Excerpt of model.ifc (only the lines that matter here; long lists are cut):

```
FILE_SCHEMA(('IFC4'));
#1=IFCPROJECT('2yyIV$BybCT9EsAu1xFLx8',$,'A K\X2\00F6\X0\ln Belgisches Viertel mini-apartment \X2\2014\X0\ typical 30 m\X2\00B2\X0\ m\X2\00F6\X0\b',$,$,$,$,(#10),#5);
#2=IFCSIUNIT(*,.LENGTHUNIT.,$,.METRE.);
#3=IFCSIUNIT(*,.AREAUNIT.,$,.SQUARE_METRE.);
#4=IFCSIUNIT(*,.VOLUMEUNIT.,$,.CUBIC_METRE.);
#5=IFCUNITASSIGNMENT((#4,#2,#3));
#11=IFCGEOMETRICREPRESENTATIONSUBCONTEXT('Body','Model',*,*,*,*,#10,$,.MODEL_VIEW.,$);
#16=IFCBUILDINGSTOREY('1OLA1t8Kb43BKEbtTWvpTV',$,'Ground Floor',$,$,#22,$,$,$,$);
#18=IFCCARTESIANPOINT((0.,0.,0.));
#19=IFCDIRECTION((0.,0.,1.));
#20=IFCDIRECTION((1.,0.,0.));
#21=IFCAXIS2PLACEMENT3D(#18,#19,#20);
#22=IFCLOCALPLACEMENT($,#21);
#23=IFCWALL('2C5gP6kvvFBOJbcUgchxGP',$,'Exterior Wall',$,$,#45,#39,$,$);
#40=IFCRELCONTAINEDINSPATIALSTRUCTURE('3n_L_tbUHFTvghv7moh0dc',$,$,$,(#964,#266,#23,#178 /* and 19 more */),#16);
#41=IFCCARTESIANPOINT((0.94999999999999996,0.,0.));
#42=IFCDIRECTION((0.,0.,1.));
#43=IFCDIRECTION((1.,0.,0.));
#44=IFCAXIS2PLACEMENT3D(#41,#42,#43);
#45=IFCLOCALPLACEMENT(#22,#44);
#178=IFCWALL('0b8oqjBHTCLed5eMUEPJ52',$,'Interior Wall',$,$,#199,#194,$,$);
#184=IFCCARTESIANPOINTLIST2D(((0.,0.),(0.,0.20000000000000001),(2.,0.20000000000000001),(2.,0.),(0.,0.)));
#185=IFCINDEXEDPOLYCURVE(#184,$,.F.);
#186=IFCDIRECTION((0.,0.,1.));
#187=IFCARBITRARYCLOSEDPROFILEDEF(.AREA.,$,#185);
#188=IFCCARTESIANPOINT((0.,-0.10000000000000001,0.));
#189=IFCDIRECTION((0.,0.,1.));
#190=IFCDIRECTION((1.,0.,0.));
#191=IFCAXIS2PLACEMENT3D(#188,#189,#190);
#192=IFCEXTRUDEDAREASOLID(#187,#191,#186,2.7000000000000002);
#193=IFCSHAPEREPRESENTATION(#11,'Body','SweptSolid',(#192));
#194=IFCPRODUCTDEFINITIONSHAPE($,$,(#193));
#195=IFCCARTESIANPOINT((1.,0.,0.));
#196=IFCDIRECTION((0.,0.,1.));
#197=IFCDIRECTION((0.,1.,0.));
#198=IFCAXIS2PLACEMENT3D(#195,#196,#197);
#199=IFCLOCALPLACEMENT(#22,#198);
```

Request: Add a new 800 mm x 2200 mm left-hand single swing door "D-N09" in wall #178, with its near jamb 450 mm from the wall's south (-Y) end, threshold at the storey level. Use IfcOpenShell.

```python
import numpy as np
import ifcopenshell
import ifcopenshell.api.feature
import ifcopenshell.api.geometry
import ifcopenshell.api.root
import ifcopenshell.api.spatial
import ifcopenshell.geom
import ifcopenshell.util.element
import ifcopenshell.util.placement
import ifcopenshell.util.representation
import ifcopenshell.util.shape
import ifcopenshell.util.unit

model = ifcopenshell.open("model.ifc")
unit_scale = ifcopenshell.util.unit.calculate_unit_scale(model)
settings = ifcopenshell.geom.settings()


def volume(element):
    """Net volume in cubic metres, openings subtracted."""
    shape = ifcopenshell.geom.create_shape(settings, element)
    return ifcopenshell.util.shape.get_volume(shape.geometry)


wall = model.by_id(178)
storey = ifcopenshell.util.element.get_container(wall, ifc_class="IfcBuildingStorey")
context = ifcopenshell.util.representation.get_context(model, "Model", "Body", "MODEL_VIEW")
before = volume(wall)

width, height, from_end, sill = 0.8, 2.2, 0.45, 0.0  # metres

# The wall runs along its own X axis, and the end named is its -X end.
wall_shape = ifcopenshell.geom.create_shape(settings, wall)
x, y, z = ifcopenshell.util.shape.get_vertices(wall_shape.geometry).T
start = x.min() + from_end
face, thickness = float(y.min()), float(y.max() - y.min())
wall_matrix = ifcopenshell.util.placement.get_local_placement(wall.ObjectPlacement)
level = ifcopenshell.util.placement.get_local_placement(storey.ObjectPlacement)[2, 3]


def in_wall(x, y):
    """Placement at x, y metres in the wall's axes, at sill height."""
    matrix = wall_matrix.copy()
    matrix[:, 3] = wall_matrix @ np.array([x / unit_scale, y / unit_scale, 0.0, 1.0])
    matrix[2, 3] = level + sill / unit_scale
    return matrix


# Opening: a box that overshoots both wall faces by 50 mm.
opening = ifcopenshell.api.root.create_entity(model, ifc_class="IfcOpeningElement", predefined_type="OPENING")
box = ifcopenshell.api.geometry.add_wall_representation(
    model, context=context, length=width, height=height, thickness=thickness + 0.1
)
ifcopenshell.api.geometry.assign_representation(model, product=opening, representation=box)
ifcopenshell.api.geometry.edit_object_placement(model, product=opening, matrix=in_wall(start, face - 0.05), is_si=False)
ifcopenshell.api.feature.add_feature(model, feature=opening, element=wall)

door = ifcopenshell.api.root.create_entity(model, ifc_class="IfcDoor", name="D-N09", predefined_type="DOOR")
door.OverallWidth, door.OverallHeight = width / unit_scale, height / unit_scale
door.OperationType = "SINGLE_SWING_LEFT"
body = ifcopenshell.api.geometry.add_door_representation(
    model,
    context=context,
    overall_width=door.OverallWidth,
    overall_height=door.OverallHeight,
    operation_type="SINGLE_SWING_LEFT",
    lining_properties={"LiningDepth": thickness / unit_scale, "ThresholdDepth": thickness / unit_scale},
)
ifcopenshell.api.geometry.assign_representation(model, product=door, representation=body)
ifcopenshell.api.spatial.assign_container(model, products=[door], relating_structure=storey)
ifcopenshell.api.feature.add_filling(model, opening=opening, element=door)

# The lining spans the wall, so the door starts at the wall face.
ifcopenshell.api.geometry.edit_object_placement(model, product=door, matrix=in_wall(start, face), is_si=False)

after = volume(wall)

print(f"wall volume {before:.3f} -> {after:.3f} m3")

model.write("model_v2.ifc")
```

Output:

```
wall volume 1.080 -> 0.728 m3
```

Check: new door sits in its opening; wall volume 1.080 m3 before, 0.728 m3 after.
